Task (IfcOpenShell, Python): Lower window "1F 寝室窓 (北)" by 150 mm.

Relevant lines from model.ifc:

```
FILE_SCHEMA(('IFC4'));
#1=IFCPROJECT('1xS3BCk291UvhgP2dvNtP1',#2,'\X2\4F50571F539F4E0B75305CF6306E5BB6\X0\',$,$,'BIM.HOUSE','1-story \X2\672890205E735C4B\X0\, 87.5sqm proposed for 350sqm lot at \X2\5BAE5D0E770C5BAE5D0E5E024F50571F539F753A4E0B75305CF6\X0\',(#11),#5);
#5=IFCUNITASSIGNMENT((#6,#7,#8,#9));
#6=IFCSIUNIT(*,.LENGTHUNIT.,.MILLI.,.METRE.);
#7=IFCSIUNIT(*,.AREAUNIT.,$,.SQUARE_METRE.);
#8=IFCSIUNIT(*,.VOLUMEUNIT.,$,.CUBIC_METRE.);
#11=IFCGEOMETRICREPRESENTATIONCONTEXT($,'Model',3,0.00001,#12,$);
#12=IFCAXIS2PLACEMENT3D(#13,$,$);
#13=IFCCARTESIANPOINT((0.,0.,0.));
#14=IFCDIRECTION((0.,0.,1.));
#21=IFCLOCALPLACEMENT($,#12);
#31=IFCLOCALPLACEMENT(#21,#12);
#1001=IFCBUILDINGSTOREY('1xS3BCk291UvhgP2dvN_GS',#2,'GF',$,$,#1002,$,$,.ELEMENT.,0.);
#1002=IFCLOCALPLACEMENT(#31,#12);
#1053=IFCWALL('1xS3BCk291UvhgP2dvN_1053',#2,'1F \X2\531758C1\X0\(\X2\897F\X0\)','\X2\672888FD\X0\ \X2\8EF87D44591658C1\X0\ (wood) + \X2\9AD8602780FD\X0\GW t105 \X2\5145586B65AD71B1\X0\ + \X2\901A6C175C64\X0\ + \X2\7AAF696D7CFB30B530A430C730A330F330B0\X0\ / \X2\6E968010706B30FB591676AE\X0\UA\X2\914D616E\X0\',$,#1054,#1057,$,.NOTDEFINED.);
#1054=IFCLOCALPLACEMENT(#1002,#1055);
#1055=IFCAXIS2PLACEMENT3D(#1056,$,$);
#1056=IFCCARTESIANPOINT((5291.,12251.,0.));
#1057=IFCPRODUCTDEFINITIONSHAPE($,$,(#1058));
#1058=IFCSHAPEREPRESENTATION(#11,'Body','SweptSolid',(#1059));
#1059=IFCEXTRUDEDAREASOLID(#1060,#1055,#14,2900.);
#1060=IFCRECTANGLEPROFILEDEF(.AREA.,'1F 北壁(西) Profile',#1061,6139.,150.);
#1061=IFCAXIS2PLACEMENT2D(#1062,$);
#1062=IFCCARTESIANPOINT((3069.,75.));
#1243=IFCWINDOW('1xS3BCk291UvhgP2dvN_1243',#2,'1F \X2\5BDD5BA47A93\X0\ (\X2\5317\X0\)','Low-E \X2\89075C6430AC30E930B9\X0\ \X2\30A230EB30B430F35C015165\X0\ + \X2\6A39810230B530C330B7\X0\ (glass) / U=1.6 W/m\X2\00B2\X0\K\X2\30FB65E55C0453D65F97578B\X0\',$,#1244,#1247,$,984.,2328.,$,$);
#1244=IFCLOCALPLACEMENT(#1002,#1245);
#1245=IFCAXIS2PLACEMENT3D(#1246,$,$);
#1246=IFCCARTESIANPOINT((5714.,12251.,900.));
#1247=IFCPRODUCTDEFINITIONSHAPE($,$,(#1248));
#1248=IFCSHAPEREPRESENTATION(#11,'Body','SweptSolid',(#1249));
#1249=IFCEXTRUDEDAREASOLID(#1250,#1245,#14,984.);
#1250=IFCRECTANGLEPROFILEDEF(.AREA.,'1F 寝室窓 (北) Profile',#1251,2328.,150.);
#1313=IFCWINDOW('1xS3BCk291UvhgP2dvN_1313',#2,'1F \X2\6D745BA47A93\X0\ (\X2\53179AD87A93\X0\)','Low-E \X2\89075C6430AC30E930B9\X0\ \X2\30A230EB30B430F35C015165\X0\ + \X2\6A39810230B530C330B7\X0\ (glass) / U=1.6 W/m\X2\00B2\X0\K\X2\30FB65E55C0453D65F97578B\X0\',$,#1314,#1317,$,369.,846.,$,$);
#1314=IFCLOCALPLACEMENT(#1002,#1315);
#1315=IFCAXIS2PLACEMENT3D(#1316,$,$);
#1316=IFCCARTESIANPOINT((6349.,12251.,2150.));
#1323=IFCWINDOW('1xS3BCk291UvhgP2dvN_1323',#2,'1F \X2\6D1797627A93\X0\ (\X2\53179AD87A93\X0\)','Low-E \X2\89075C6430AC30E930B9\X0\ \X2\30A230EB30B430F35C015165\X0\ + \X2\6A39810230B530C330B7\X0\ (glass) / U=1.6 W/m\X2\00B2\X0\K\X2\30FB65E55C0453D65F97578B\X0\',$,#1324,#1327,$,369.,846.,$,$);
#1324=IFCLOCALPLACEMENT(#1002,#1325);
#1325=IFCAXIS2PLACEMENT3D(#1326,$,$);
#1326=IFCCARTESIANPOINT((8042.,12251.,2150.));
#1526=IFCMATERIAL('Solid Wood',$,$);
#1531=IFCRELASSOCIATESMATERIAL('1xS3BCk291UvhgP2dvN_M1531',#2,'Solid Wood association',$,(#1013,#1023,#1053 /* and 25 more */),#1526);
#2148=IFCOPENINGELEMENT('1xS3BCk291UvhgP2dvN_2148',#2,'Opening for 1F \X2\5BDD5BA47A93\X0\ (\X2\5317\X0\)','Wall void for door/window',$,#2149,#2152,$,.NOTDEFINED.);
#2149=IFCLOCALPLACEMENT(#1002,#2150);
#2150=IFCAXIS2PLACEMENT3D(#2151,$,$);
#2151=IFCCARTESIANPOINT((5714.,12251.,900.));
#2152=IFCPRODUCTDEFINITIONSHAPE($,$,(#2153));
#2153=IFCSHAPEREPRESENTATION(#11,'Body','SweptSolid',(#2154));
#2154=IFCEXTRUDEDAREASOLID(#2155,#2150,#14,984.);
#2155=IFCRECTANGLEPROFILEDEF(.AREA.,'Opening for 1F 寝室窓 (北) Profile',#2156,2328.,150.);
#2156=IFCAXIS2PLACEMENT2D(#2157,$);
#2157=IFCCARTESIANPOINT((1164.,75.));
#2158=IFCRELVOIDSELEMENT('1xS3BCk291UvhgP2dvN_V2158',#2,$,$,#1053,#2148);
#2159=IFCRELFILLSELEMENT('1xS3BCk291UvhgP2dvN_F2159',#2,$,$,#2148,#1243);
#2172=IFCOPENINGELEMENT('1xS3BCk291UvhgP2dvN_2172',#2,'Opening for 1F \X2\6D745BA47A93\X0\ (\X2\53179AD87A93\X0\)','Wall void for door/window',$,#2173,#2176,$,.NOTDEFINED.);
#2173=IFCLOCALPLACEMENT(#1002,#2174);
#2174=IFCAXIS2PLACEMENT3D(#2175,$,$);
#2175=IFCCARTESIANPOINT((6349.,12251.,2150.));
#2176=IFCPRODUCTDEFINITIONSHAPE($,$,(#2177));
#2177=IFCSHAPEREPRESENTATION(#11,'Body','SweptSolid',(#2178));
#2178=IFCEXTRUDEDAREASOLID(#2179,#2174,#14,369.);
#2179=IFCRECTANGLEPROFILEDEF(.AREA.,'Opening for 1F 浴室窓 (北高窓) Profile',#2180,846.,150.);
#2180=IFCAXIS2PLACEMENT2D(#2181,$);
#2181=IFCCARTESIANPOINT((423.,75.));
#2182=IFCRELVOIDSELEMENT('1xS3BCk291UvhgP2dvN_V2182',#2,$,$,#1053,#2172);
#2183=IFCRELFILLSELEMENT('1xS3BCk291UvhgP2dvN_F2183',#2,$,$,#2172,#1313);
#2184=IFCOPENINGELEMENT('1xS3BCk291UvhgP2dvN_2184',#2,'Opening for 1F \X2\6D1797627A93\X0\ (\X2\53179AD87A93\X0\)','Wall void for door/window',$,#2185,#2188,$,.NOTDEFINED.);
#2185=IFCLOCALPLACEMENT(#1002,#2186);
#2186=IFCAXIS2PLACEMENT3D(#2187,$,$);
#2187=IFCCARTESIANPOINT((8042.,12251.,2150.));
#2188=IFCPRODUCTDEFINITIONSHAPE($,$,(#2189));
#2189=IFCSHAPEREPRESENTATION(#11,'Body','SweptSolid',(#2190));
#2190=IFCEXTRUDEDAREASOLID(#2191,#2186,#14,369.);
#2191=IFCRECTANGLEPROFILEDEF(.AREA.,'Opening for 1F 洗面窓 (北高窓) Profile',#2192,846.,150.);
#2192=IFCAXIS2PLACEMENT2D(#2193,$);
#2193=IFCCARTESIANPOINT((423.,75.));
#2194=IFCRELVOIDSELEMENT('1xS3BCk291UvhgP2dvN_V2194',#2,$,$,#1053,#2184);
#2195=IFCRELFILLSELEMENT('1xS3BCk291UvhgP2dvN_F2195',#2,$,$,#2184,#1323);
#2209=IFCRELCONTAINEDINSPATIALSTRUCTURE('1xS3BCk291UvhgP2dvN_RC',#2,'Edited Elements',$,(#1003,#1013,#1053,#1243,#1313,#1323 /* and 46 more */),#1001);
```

```python
import numpy as np
import ifcopenshell
import ifcopenshell.api.geometry
import ifcopenshell.util.placement
import ifcopenshell.util.unit

model = ifcopenshell.open("model.ifc")
unit_scale = ifcopenshell.util.unit.calculate_unit_scale(model)

window = model.by_guid("1xS3BCk291UvhgP2dvN_1243")
opening = window.FillsVoids[0].RelatingOpeningElement
dz = -0.15 / unit_scale

shift = np.array([0.0, 0.0, dz])
# The window is not placed relative to its opening, so move both.
for product in (opening, window):
    matrix = ifcopenshell.util.placement.get_local_placement(product.ObjectPlacement)
    matrix[:3, 3] += shift
    ifcopenshell.api.geometry.edit_object_placement(model, product=product, matrix=matrix, is_si=False)

print(f"moved by {dz * unit_scale:+.3f} m")

model.write("model-out.ifc")
```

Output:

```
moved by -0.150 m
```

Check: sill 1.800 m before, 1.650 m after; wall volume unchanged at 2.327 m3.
